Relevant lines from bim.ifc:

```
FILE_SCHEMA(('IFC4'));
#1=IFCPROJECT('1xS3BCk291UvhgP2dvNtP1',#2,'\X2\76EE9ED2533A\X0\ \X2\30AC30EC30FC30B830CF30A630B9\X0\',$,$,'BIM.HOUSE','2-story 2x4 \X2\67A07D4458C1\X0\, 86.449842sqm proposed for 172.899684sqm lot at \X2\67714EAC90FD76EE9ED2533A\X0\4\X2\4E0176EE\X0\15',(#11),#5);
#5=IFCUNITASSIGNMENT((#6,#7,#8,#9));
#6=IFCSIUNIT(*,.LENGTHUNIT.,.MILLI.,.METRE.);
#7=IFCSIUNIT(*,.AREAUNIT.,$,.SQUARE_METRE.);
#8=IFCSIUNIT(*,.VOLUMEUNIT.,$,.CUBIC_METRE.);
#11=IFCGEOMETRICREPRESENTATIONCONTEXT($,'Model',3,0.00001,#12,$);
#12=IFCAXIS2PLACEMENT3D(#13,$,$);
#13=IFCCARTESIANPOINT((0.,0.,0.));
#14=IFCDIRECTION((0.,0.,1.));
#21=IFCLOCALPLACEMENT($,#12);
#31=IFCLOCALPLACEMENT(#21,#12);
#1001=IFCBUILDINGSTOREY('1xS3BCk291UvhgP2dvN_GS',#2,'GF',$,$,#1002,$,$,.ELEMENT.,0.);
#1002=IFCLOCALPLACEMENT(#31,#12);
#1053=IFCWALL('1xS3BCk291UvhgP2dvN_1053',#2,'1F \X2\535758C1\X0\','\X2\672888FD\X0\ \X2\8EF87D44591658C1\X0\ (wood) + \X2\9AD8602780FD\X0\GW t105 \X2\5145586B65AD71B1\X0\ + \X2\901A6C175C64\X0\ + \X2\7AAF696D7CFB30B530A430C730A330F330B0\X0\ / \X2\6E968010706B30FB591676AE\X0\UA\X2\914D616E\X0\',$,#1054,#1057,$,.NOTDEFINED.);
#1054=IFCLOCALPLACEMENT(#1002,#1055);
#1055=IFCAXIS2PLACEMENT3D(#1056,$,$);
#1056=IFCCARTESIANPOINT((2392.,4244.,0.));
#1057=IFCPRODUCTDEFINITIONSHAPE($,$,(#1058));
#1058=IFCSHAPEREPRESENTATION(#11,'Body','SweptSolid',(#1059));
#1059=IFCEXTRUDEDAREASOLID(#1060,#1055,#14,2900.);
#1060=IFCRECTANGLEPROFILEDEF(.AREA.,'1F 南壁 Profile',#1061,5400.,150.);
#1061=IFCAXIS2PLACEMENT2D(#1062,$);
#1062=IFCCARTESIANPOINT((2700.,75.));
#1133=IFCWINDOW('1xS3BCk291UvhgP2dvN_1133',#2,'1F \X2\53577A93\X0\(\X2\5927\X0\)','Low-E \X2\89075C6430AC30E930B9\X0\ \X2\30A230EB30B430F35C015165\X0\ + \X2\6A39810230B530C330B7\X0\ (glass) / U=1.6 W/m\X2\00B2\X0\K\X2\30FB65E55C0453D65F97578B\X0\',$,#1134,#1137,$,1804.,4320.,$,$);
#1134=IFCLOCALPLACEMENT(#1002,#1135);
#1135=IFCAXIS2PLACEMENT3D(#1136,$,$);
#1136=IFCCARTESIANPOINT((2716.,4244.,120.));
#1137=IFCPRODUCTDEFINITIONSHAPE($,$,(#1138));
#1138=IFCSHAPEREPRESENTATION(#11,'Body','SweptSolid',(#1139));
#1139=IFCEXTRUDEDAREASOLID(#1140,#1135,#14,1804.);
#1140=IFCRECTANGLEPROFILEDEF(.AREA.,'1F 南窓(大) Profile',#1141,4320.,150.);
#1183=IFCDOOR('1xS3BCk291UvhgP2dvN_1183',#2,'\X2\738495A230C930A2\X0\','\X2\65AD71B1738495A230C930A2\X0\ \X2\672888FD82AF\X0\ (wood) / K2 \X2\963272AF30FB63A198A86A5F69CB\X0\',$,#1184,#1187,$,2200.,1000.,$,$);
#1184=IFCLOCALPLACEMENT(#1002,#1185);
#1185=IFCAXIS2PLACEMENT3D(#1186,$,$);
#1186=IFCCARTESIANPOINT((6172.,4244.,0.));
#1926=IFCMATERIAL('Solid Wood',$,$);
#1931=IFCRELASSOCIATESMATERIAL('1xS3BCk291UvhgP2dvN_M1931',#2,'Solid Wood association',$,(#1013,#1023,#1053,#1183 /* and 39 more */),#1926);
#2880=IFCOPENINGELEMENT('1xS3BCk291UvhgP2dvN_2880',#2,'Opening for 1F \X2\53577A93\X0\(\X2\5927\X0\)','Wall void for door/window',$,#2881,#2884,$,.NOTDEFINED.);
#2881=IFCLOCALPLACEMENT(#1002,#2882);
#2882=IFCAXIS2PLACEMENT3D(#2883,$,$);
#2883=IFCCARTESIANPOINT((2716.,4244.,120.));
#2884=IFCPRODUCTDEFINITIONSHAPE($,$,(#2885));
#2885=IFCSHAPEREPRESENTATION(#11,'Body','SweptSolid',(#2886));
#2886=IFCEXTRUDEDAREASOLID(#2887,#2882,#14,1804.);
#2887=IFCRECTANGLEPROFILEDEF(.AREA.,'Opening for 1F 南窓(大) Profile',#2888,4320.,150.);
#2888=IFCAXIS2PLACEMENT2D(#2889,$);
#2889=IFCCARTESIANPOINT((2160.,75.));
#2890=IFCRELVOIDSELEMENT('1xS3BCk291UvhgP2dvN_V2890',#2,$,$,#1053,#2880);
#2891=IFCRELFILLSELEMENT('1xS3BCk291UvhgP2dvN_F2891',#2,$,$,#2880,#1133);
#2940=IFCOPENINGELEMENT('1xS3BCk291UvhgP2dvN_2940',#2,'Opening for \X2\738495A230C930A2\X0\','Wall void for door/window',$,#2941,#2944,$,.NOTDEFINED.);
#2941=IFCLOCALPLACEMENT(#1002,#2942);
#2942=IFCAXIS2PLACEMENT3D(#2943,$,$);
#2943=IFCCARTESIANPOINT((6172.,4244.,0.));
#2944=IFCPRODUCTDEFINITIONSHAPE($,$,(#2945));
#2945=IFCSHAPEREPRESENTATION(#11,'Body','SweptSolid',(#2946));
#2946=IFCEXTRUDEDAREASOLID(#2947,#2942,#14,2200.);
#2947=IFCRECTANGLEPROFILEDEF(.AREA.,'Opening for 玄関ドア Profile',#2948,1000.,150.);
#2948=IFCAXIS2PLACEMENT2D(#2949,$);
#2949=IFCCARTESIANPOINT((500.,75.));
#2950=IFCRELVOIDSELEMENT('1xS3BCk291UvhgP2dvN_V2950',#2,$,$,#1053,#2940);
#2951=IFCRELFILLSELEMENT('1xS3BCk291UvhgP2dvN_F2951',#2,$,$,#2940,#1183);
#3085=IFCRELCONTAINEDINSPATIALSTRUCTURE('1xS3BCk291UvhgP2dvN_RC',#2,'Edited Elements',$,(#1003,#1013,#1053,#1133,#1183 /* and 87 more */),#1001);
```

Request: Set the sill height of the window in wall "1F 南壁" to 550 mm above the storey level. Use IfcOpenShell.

```python
import numpy as np
import ifcopenshell
import ifcopenshell.api.geometry
import ifcopenshell.geom
import ifcopenshell.util.element
import ifcopenshell.util.placement
import ifcopenshell.util.shape
import ifcopenshell.util.unit

model = ifcopenshell.open("bim.ifc")
unit_scale = ifcopenshell.util.unit.calculate_unit_scale(model)

window = model.by_guid("1xS3BCk291UvhgP2dvN_1133")
opening = window.FillsVoids[0].RelatingOpeningElement
storey = ifcopenshell.util.element.get_container(window, ifc_class="IfcBuildingStorey")
level = ifcopenshell.util.placement.get_local_placement(storey.ObjectPlacement)[2, 3]

# The opening's origin need not be at the sill, so measure its lowest point.
shape = ifcopenshell.geom.create_shape(ifcopenshell.geom.settings(), opening)
bottom = ifcopenshell.util.shape.get_shape_bottom_elevation(shape, shape.geometry) / unit_scale
dz = level + 550.0 - bottom

shift = np.array([0.0, 0.0, dz])
# The window is not placed relative to its opening, so move both.
for product in (opening, window):
    matrix = ifcopenshell.util.placement.get_local_placement(product.ObjectPlacement)
    matrix[:3, 3] += shift
    ifcopenshell.api.geometry.edit_object_placement(model, product=product, matrix=matrix, is_si=False)

print(f"moved by {dz * unit_scale:+.3f} m")

model.write("bim_edited.ifc")
```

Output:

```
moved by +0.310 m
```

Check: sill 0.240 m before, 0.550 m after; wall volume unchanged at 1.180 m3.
